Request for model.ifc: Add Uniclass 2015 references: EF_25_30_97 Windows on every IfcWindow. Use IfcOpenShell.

First a look at what the model holds.

```python
import ifcopenshell

model = ifcopenshell.open("model.ifc")
print(model.schema)
print("classifications:", [c.Name for c in model.by_type("IfcClassification")])
for ifc_class in ("IfcDoor", "IfcRoof", "IfcStair", "IfcWall", "IfcWindow"):
    print(ifc_class, len(model.by_type(ifc_class)))
```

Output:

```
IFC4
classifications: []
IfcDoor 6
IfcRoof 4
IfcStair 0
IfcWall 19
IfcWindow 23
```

```python
import ifcopenshell
import ifcopenshell.api.classification

model = ifcopenshell.open("model.ifc")

system = ifcopenshell.api.classification.add_classification(model, classification="Uniclass 2015")

codes = {
    "IfcWindow": ("EF_25_30_97", "Windows"),
}
for ifc_class, (code, name) in codes.items():
    products = model.by_type(ifc_class)
    ifcopenshell.api.classification.add_reference(
        model, products=products, classification=system, identification=code, name=name
    )
    print(code, len(products))

model.write("model_edited.ifc")
```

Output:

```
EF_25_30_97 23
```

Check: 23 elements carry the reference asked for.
